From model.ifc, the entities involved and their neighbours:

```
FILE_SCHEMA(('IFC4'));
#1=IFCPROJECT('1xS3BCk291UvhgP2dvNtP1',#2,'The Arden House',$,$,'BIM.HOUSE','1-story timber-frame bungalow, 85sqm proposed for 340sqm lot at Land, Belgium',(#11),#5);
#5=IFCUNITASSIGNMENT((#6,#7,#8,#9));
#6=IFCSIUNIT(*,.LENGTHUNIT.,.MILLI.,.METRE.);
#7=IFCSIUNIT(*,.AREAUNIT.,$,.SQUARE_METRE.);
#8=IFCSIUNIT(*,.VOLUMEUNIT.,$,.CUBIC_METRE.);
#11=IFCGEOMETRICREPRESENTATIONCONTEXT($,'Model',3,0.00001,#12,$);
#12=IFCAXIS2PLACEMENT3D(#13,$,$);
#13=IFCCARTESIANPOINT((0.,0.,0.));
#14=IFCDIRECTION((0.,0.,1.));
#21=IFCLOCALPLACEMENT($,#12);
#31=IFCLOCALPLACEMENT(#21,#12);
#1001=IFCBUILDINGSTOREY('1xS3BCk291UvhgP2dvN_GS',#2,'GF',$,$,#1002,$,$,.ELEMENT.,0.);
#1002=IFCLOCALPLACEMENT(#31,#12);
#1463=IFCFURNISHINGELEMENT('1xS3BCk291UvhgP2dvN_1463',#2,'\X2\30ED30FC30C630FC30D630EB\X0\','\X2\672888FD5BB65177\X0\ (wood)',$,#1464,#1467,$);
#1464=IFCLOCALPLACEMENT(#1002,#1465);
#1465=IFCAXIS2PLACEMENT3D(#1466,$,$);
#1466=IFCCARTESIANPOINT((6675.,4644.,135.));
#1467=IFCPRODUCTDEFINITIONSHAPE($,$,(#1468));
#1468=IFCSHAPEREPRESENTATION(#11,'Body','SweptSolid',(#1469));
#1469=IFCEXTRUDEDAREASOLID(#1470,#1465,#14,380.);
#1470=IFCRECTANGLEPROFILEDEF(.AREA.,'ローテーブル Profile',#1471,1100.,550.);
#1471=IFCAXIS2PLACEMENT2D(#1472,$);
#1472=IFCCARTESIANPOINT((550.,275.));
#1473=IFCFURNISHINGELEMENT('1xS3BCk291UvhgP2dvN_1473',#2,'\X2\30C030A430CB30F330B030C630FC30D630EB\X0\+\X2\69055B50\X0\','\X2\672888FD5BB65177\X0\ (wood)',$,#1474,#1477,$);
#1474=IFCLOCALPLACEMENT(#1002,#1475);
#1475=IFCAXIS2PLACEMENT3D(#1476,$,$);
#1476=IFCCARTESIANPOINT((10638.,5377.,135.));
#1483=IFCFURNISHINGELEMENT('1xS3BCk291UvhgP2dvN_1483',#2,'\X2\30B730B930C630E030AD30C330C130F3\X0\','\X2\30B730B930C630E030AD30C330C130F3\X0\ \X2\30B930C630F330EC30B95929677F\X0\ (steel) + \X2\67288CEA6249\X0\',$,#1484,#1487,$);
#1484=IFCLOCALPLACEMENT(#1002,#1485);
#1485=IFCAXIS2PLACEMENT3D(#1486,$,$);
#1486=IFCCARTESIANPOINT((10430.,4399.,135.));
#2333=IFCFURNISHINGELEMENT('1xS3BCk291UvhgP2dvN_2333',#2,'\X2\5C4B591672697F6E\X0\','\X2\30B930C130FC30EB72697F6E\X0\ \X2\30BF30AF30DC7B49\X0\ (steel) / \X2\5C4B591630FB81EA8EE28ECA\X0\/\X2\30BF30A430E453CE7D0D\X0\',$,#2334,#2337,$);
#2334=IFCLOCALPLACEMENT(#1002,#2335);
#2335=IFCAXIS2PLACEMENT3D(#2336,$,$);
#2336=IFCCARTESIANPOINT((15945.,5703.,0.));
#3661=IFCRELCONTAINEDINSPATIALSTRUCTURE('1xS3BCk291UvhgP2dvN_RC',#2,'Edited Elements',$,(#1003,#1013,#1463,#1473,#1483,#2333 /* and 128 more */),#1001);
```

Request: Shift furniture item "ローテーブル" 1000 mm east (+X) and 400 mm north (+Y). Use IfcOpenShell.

```python
import ifcopenshell
import ifcopenshell.api.geometry
import ifcopenshell.util.placement
import ifcopenshell.util.unit

model = ifcopenshell.open("model.ifc")
unit_scale = ifcopenshell.util.unit.calculate_unit_scale(model)

item = model.by_id(1463)
matrix = ifcopenshell.util.placement.get_local_placement(item.ObjectPlacement)
matrix[0, 3] += 1 / unit_scale
matrix[1, 3] += 0.4 / unit_scale
ifcopenshell.api.geometry.edit_object_placement(model, product=item, matrix=matrix, is_si=False)

print(ifcopenshell.util.placement.get_local_placement(item.ObjectPlacement).round(3) + 0.0)

model.write("model_edited.ifc")
```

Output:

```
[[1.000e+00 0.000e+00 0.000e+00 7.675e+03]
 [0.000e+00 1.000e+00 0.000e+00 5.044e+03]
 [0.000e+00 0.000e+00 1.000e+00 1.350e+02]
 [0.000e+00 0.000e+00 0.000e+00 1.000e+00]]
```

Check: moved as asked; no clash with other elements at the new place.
